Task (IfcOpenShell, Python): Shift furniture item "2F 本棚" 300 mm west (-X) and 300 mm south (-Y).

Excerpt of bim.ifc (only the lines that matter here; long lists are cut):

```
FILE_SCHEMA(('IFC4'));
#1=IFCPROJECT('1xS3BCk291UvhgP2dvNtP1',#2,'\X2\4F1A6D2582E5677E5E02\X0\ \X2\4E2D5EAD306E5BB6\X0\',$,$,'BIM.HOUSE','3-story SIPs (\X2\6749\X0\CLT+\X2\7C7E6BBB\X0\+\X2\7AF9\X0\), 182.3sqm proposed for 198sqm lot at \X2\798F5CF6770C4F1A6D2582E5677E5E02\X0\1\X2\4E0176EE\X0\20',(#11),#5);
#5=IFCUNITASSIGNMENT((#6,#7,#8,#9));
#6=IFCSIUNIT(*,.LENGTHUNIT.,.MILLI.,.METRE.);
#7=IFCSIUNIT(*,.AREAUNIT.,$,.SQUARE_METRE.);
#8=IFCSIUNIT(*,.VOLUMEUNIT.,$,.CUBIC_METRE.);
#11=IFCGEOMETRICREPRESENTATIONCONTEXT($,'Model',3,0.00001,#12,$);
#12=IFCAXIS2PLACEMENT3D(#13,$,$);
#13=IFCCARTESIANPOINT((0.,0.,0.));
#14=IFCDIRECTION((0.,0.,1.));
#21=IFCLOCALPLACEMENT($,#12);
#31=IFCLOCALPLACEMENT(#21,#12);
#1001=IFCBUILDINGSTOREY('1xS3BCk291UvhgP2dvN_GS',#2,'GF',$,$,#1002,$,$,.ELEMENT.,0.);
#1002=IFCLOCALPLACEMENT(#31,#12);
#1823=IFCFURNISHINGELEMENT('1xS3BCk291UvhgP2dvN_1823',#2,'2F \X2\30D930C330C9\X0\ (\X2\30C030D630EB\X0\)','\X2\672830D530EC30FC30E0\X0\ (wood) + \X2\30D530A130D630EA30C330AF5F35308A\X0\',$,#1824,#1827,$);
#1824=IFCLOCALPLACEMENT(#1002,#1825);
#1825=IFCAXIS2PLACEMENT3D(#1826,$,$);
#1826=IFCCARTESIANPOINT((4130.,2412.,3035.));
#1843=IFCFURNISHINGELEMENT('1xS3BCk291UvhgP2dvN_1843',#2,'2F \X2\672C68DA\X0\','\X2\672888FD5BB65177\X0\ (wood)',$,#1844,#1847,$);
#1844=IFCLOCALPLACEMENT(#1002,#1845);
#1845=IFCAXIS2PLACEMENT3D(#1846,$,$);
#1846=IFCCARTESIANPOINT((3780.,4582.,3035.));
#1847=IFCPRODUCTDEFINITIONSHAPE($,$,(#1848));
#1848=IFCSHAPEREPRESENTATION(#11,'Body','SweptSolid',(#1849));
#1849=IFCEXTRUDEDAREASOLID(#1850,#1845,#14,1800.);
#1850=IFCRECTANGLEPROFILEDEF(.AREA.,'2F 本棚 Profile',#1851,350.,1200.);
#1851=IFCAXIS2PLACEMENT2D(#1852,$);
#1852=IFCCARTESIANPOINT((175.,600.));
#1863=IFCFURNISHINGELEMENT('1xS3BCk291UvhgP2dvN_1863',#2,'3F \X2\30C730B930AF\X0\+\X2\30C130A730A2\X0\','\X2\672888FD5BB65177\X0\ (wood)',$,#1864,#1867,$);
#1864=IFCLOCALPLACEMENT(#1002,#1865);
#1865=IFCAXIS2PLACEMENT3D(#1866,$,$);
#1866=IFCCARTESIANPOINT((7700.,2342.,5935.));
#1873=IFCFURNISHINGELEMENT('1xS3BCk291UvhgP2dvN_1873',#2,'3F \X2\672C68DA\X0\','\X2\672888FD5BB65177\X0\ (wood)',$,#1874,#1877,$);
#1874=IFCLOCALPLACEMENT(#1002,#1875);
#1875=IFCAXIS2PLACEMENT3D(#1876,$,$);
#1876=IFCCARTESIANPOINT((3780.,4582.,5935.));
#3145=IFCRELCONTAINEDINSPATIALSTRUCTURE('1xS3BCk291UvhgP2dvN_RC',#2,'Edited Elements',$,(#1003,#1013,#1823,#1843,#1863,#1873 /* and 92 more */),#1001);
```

```python
import ifcopenshell
import ifcopenshell.api.geometry
import ifcopenshell.util.placement

model = ifcopenshell.open("bim.ifc")

item = model.by_id(1843)
matrix = ifcopenshell.util.placement.get_local_placement(item.ObjectPlacement)
matrix[0, 3] -= 300.0
matrix[1, 3] -= 300.0
ifcopenshell.api.geometry.edit_object_placement(model, product=item, matrix=matrix, is_si=False)

print(ifcopenshell.util.placement.get_local_placement(item.ObjectPlacement).round(3) + 0.0)

model.write("bim_edited.ifc")
```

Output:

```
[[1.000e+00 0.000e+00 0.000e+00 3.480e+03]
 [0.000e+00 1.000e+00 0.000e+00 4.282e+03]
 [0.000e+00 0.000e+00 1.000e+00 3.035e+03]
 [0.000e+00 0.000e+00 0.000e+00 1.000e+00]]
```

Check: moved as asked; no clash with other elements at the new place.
